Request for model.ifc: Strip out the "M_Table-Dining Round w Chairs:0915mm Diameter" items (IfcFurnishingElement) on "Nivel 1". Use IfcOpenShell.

First a look at what the model holds.

```python
import ifcopenshell
import ifcopenshell.util.element

model = ifcopenshell.open("model.ifc")
print(model.schema)
storey = next(s for s in model.by_type("IfcBuildingStorey") if s.Name == "Nivel 1")
furniture = [e for e in ifcopenshell.util.element.get_decomposition(storey) if e.is_a("IfcFurnishingElement")]
seen = {}
for e in furniture:
    element_type = ifcopenshell.util.element.get_type(e)
    name = element_type.Name if element_type not in (None, e) else None
    seen[name] = seen.get(name, 0) + 1
for name, count in sorted(seen.items(), key=str):
    print(count, "x", name)
```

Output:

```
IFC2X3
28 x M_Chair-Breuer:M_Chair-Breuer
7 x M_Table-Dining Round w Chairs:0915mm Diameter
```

```python
import ifcopenshell
import ifcopenshell.api.root
import ifcopenshell.util.element

model = ifcopenshell.open("model.ifc")

storey = next(s for s in model.by_type("IfcBuildingStorey") if s.Name == "Nivel 1")
furniture = [e for e in ifcopenshell.util.element.get_decomposition(storey) if e.is_a("IfcFurnishingElement")]
targets = [e for e in furniture if (t := ifcopenshell.util.element.get_type(e)) not in (None, e) and t.Name == "M_Table-Dining Round w Chairs:0915mm Diameter"]

for e in targets:
    ifcopenshell.api.root.remove_product(model, product=e)
print(len(targets), "removed")

model.write("model_v2.ifc")
```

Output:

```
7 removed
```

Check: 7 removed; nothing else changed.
